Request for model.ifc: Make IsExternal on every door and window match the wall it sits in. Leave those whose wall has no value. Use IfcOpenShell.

First a look at what the model holds.

```python
import ifcopenshell
import ifcopenshell.util.element

model = ifcopenshell.open("model.ifc")
print(model.schema)
seen = {}
for e in model.by_type("IfcDoor") + model.by_type("IfcWindow"):
    if not e.FillsVoids:
        continue
    host = e.FillsVoids[0].RelatingOpeningElement.VoidsElements[0].RelatingBuildingElement
    own = ifcopenshell.util.element.get_pset(e, f"Pset_{e.is_a()[3:].removesuffix('StandardCase')}Common", "IsExternal")
    wall = ifcopenshell.util.element.get_pset(host, "Pset_WallCommon", "IsExternal")
    seen[e.is_a(), own, wall] = seen.get((e.is_a(), own, wall), 0) + 1
for (cls, own, wall), count in sorted(seen.items(), key=str):
    print(count, cls, "IsExternal:", own, "| host wall:", wall)
```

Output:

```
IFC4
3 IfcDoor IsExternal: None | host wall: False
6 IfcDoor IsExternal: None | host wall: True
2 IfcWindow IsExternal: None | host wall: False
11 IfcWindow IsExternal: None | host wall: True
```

```python
import ifcopenshell
import ifcopenshell.api.pset
import ifcopenshell.util.element

model = ifcopenshell.open("model.ifc")

count = 0
for ifc_class, pset_name in (("IfcDoor", "Pset_DoorCommon"), ("IfcWindow", "Pset_WindowCommon")):
    for e in model.by_type(ifc_class):
        if not e.FillsVoids:
            continue
        host = e.FillsVoids[0].RelatingOpeningElement.VoidsElements[0].RelatingBuildingElement
        external = ifcopenshell.util.element.get_pset(host, "Pset_WallCommon", "IsExternal")
        if external is None or ifcopenshell.util.element.get_pset(e, pset_name, "IsExternal") == external:
            continue
        pset = ifcopenshell.api.pset.add_pset(model, product=e, name=pset_name)
        ifcopenshell.api.pset.edit_pset(model, pset=pset, properties={"IsExternal": external})
        count += 1

print(count, "updated")

model.write("model_v2.ifc")
```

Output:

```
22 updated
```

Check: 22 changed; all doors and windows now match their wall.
